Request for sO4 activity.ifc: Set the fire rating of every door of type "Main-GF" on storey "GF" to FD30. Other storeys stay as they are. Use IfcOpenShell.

First a look at what the model holds.

```python
import ifcopenshell
import ifcopenshell.util.element

model = ifcopenshell.open("sO4 activity.ifc")
print(model.schema)
storey = next(s for s in model.by_type("IfcBuildingStorey") if s.Name == "GF")
doors = [e for e in ifcopenshell.util.element.get_decomposition(storey) if e.is_a("IfcDoor")]
seen = {}
for e in doors:
    element_type = ifcopenshell.util.element.get_type(e)
    key = (element_type.Name if element_type != e and element_type else None, ifcopenshell.util.element.get_pset(e, "Pset_DoorCommon", "FireRating"))
    seen[key] = seen.get(key, 0) + 1
for (name, value), count in sorted(seen.items(), key=str):
    print(count, "x", name, "|", value)
```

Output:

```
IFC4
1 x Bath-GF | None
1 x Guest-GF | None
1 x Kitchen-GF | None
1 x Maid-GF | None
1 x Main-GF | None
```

```python
import ifcopenshell
import ifcopenshell.api.pset
import ifcopenshell.util.element

model = ifcopenshell.open("sO4 activity.ifc")

storey = next(s for s in model.by_type("IfcBuildingStorey") if s.Name == "GF")
doors = [e for e in ifcopenshell.util.element.get_decomposition(storey) if e.is_a("IfcDoor")]

count = 0
for e in doors:
    element_type = ifcopenshell.util.element.get_type(e)
    if element_type in (None, e) or element_type.Name != "Main-GF":
        continue
    # add_pset returns the element's existing set when there is one.
    pset = ifcopenshell.api.pset.add_pset(model, product=e, name="Pset_DoorCommon")
    ifcopenshell.api.pset.edit_pset(model, pset=pset, properties={"FireRating": "FD30"})
    count += 1

print(count, "doors updated")

model.write("sO4 activity_rev.ifc")
```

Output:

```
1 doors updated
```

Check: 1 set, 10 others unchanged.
